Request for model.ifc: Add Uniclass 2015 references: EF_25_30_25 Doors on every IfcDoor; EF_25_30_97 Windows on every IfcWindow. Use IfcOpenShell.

First a look at what the model holds.

```python
import ifcopenshell

model = ifcopenshell.open("model.ifc")
print(model.schema)
print("classifications:", [c.Name for c in model.by_type("IfcClassification")])
for ifc_class in ("IfcDoor", "IfcRoof", "IfcStair", "IfcWall", "IfcWindow"):
    print(ifc_class, len(model.by_type(ifc_class)))
```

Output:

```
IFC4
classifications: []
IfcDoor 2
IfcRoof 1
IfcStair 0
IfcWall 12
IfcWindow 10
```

```python
import ifcopenshell
import ifcopenshell.api.classification

model = ifcopenshell.open("model.ifc")

system = ifcopenshell.api.classification.add_classification(model, classification="Uniclass 2015")

codes = {
    "IfcDoor": ("EF_25_30_25", "Doors"),
    "IfcWindow": ("EF_25_30_97", "Windows"),
}
for ifc_class, (code, name) in codes.items():
    products = model.by_type(ifc_class)
    ifcopenshell.api.classification.add_reference(
        model, products=products, classification=system, identification=code, name=name
    )
    print(code, len(products))

model.write("model_v2.ifc")
```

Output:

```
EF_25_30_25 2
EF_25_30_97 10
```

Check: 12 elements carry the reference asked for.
